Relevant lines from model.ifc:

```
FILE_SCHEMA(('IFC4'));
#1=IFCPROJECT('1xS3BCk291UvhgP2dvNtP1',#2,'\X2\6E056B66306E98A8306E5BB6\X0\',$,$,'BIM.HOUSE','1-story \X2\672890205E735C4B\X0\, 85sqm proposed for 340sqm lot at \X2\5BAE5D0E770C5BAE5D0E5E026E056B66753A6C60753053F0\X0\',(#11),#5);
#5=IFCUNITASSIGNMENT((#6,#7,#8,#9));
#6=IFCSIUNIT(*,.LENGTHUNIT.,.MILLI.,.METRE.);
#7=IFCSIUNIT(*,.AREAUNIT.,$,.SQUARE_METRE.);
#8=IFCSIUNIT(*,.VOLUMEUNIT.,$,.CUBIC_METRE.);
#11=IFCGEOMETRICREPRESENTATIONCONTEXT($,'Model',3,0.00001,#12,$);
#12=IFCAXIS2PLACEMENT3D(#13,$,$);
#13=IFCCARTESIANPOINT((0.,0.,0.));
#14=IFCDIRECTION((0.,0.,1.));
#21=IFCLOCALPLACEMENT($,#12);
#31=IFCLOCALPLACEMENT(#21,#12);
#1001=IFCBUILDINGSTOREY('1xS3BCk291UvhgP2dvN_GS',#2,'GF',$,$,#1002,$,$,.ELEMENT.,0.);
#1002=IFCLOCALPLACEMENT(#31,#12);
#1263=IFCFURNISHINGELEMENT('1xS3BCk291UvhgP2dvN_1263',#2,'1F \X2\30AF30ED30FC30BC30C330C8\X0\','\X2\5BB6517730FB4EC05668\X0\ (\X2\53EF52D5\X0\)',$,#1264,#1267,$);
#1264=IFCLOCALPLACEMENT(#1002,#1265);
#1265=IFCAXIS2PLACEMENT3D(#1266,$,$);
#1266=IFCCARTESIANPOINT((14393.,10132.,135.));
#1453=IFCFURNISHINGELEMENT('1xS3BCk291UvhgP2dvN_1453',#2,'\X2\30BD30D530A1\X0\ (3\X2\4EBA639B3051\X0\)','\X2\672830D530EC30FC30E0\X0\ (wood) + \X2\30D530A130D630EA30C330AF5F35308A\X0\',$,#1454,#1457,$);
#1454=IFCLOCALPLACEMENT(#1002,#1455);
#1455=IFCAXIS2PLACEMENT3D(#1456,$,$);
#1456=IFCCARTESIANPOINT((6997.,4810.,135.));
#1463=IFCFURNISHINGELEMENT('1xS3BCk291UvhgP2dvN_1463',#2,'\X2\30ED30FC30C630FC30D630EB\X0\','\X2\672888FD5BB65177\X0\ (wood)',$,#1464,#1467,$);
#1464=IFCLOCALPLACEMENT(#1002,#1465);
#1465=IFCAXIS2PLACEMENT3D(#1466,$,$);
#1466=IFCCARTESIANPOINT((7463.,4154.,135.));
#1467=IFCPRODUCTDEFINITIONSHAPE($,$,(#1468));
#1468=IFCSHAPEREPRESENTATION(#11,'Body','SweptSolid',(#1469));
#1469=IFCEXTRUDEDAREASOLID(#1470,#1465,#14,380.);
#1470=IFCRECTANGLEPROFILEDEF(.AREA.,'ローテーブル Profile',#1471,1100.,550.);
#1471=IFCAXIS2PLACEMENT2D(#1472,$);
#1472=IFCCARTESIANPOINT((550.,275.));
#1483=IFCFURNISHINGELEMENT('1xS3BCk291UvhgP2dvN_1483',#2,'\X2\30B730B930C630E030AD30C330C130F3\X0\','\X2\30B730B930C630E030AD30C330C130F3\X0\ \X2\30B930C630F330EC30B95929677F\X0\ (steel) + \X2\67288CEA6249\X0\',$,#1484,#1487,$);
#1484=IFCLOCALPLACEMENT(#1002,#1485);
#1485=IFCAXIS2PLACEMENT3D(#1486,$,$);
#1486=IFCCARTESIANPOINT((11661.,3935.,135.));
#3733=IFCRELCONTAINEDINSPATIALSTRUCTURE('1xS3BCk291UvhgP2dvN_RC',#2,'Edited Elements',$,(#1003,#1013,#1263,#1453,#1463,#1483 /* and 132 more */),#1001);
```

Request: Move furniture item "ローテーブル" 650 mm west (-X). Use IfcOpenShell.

```python
import ifcopenshell
import ifcopenshell.api.geometry
import ifcopenshell.util.placement

model = ifcopenshell.open("model.ifc")

item = model.by_id(1463)
matrix = ifcopenshell.util.placement.get_local_placement(item.ObjectPlacement)
matrix[0, 3] -= 650.0
ifcopenshell.api.geometry.edit_object_placement(model, product=item, matrix=matrix, is_si=False)

print(ifcopenshell.util.placement.get_local_placement(item.ObjectPlacement).round(3) + 0.0)

model.write("model_rev.ifc")
```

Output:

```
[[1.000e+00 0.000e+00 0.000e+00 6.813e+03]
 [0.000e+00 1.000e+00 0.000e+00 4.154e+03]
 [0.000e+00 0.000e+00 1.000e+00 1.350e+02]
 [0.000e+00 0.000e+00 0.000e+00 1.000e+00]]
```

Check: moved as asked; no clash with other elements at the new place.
